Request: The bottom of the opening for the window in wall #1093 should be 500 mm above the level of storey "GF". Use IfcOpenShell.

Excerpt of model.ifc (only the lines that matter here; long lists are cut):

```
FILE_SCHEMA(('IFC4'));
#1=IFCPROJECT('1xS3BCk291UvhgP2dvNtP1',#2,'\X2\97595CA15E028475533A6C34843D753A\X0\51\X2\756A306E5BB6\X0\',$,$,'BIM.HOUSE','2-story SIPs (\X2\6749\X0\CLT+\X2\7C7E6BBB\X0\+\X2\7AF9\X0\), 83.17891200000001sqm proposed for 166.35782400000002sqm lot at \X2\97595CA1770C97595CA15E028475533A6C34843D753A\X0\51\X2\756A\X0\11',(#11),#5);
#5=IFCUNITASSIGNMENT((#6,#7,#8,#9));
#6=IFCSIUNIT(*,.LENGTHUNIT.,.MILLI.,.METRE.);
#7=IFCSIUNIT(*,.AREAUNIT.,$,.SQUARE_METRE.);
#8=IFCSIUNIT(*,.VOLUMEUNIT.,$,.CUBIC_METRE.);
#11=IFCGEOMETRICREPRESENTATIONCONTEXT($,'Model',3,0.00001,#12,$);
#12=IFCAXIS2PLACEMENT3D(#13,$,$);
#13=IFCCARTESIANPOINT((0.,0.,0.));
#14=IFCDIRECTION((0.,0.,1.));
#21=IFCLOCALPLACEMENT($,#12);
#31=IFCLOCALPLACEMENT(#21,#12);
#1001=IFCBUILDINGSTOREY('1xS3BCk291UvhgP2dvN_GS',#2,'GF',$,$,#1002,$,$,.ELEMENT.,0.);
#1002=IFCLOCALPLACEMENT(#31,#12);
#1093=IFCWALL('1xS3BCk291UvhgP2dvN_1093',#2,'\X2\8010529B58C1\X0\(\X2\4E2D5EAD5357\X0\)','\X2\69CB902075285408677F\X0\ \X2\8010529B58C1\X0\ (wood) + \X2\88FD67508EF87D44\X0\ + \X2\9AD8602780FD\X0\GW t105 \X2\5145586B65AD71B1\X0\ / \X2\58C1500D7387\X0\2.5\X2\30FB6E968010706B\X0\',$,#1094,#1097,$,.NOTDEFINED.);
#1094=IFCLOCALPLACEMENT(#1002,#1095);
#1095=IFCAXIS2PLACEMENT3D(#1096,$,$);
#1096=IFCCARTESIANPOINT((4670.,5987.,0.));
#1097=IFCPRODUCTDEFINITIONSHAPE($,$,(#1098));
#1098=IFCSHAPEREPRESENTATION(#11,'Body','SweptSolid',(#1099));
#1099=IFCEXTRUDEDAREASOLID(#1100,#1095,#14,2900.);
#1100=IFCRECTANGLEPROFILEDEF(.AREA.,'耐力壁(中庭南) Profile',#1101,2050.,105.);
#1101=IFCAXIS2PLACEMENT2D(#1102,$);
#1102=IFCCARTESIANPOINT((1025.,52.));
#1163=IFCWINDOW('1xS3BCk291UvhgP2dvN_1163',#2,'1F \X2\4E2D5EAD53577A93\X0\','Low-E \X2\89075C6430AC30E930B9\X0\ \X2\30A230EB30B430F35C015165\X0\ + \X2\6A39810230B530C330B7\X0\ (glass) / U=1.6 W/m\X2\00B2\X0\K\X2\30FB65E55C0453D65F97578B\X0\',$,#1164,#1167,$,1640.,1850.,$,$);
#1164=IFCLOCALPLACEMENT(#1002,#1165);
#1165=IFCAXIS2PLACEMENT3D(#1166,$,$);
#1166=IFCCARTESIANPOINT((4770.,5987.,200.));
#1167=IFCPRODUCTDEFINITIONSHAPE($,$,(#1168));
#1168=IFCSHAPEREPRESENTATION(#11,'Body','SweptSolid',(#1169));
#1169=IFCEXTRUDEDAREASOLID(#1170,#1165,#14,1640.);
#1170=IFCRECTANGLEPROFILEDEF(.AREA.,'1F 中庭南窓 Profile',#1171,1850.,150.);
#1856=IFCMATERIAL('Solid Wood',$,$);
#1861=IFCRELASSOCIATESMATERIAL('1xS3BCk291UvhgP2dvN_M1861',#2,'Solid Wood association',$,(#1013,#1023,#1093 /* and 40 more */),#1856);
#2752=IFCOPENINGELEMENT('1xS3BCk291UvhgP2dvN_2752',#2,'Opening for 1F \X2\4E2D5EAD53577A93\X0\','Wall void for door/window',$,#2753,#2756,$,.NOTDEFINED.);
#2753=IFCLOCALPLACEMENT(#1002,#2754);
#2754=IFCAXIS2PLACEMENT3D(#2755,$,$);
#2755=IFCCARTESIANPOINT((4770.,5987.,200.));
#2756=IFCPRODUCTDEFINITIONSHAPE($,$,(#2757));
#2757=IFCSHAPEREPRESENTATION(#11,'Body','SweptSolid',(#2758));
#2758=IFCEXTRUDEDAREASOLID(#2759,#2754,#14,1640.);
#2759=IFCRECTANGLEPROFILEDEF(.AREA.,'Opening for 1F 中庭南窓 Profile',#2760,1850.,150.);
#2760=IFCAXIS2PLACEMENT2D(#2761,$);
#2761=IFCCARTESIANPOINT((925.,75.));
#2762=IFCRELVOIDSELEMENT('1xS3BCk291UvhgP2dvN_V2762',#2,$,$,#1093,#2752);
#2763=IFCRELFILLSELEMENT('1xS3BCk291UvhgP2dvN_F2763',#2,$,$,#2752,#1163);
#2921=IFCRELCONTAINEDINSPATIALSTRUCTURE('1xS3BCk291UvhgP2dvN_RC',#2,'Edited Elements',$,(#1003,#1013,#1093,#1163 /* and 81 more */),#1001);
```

```python
import numpy as np
import ifcopenshell
import ifcopenshell.api.geometry
import ifcopenshell.geom
import ifcopenshell.util.element
import ifcopenshell.util.placement
import ifcopenshell.util.shape
import ifcopenshell.util.unit

model = ifcopenshell.open("model.ifc")
unit_scale = ifcopenshell.util.unit.calculate_unit_scale(model)

window = model.by_id(1163)
opening = window.FillsVoids[0].RelatingOpeningElement
storey = ifcopenshell.util.element.get_container(window, ifc_class="IfcBuildingStorey")
level = ifcopenshell.util.placement.get_local_placement(storey.ObjectPlacement)[2, 3]

# The opening's origin need not be at the sill, so measure its lowest point.
shape = ifcopenshell.geom.create_shape(ifcopenshell.geom.settings(), opening)
bottom = ifcopenshell.util.shape.get_shape_bottom_elevation(shape, shape.geometry) / unit_scale
dz = level + 0.5 / unit_scale - bottom

shift = np.array([0.0, 0.0, dz])
# The window is not placed relative to its opening, so move both.
for product in (opening, window):
    matrix = ifcopenshell.util.placement.get_local_placement(product.ObjectPlacement)
    matrix[:3, 3] += shift
    ifcopenshell.api.geometry.edit_object_placement(model, product=product, matrix=matrix, is_si=False)

print(f"moved by {dz * unit_scale:+.3f} m")

model.write("model_edited.ifc")
```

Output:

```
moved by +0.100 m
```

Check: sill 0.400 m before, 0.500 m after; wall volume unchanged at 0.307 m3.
